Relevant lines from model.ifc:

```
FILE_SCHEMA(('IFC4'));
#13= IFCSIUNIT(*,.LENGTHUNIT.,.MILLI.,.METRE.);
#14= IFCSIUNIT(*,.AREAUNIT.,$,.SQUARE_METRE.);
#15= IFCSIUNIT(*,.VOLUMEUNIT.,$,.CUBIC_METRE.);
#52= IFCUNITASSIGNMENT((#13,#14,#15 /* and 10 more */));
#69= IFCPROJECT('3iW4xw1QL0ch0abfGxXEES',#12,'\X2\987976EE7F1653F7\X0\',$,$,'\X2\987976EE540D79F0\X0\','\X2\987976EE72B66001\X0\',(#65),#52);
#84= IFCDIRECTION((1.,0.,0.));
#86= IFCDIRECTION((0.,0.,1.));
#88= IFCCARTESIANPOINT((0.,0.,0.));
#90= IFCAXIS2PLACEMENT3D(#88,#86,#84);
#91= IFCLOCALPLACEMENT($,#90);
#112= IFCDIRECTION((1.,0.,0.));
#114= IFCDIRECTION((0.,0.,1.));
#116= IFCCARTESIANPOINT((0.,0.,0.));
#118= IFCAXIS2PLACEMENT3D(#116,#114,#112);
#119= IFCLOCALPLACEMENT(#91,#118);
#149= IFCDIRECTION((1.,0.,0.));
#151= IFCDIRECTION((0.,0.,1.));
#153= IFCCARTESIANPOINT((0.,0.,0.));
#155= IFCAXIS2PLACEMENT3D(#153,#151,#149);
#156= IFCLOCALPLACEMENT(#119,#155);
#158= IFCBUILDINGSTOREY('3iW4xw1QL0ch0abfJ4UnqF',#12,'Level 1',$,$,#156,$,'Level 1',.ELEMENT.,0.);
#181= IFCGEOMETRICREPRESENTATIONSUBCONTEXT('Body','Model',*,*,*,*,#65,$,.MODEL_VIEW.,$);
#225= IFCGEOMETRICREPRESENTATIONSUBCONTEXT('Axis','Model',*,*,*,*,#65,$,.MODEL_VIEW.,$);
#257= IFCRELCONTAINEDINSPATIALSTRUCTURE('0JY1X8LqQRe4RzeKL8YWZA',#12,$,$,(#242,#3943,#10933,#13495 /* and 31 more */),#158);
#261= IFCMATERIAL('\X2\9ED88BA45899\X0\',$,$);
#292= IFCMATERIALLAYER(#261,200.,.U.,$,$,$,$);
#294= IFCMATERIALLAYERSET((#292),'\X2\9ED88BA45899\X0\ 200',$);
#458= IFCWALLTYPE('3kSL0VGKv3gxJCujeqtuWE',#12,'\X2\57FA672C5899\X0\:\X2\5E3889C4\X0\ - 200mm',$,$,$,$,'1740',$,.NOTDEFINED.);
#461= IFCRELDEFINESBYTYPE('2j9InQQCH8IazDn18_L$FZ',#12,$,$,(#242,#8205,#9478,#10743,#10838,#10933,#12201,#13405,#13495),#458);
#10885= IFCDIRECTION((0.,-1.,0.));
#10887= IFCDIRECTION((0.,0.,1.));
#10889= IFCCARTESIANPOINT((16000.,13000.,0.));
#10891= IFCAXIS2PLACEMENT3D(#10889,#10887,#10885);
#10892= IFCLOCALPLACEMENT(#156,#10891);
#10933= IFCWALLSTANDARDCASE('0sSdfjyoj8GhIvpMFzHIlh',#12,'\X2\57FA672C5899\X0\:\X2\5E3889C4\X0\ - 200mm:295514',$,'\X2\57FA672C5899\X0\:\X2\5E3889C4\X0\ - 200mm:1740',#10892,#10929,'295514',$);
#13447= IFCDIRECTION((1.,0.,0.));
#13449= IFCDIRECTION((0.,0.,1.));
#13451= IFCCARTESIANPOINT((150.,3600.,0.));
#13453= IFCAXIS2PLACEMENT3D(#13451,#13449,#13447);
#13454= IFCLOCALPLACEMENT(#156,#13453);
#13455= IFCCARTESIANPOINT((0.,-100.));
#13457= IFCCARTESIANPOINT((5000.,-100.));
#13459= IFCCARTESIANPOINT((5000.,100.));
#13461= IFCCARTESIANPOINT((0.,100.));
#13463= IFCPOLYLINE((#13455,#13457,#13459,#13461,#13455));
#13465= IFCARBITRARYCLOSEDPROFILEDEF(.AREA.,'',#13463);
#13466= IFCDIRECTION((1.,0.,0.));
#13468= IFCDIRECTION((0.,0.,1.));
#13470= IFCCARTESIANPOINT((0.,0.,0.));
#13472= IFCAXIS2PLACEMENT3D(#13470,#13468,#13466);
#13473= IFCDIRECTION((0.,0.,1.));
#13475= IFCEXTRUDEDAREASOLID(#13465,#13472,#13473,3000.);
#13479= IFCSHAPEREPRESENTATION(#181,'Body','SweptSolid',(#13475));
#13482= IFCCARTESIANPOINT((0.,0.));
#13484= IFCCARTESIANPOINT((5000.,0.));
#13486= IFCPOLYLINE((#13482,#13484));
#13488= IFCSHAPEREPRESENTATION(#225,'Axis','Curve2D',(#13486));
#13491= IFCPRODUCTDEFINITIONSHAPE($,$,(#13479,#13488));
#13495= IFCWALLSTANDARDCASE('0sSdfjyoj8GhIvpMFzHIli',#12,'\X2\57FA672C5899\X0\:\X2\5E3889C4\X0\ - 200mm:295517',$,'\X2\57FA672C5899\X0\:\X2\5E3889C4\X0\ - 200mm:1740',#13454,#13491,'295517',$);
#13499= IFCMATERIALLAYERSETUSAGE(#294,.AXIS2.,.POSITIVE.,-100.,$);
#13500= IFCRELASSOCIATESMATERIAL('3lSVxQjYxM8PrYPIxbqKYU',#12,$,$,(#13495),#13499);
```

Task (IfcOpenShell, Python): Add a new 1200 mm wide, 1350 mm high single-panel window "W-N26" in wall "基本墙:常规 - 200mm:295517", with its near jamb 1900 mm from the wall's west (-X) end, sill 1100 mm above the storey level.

```python
import numpy as np
import ifcopenshell
import ifcopenshell.api.feature
import ifcopenshell.api.geometry
import ifcopenshell.api.root
import ifcopenshell.api.spatial
import ifcopenshell.geom
import ifcopenshell.util.element
import ifcopenshell.util.placement
import ifcopenshell.util.representation
import ifcopenshell.util.shape
import ifcopenshell.util.unit

model = ifcopenshell.open("model.ifc")
unit_scale = ifcopenshell.util.unit.calculate_unit_scale(model)
settings = ifcopenshell.geom.settings()


def volume(element):
    """Net volume in cubic metres, openings subtracted."""
    shape = ifcopenshell.geom.create_shape(settings, element)
    return ifcopenshell.util.shape.get_volume(shape.geometry)


wall = model.by_id(13495)
storey = ifcopenshell.util.element.get_container(wall, ifc_class="IfcBuildingStorey")
context = ifcopenshell.util.representation.get_context(model, "Model", "Body", "MODEL_VIEW")
before = volume(wall)

width, height, from_end, sill = 1.2, 1.35, 1.9, 1.1  # metres

# The wall runs along its own X axis, and the end named is its -X end.
wall_shape = ifcopenshell.geom.create_shape(settings, wall)
x, y, z = ifcopenshell.util.shape.get_vertices(wall_shape.geometry).T
start = x.min() + from_end
face, thickness = float(y.min()), float(y.max() - y.min())
wall_matrix = ifcopenshell.util.placement.get_local_placement(wall.ObjectPlacement)
level = ifcopenshell.util.placement.get_local_placement(storey.ObjectPlacement)[2, 3]


def in_wall(x, y):
    """Placement at x, y metres in the wall's axes, at sill height."""
    matrix = wall_matrix.copy()
    matrix[:, 3] = wall_matrix @ np.array([x / unit_scale, y / unit_scale, 0.0, 1.0])
    matrix[2, 3] = level + sill / unit_scale
    return matrix


# Opening: a box that overshoots both wall faces by 50 mm.
opening = ifcopenshell.api.root.create_entity(model, ifc_class="IfcOpeningElement", predefined_type="OPENING")
box = ifcopenshell.api.geometry.add_wall_representation(
    model, context=context, length=width, height=height, thickness=thickness + 0.1
)
ifcopenshell.api.geometry.assign_representation(model, product=opening, representation=box)
ifcopenshell.api.geometry.edit_object_placement(model, product=opening, matrix=in_wall(start, face - 0.05), is_si=False)
ifcopenshell.api.feature.add_feature(model, feature=opening, element=wall)

window = ifcopenshell.api.root.create_entity(model, ifc_class="IfcWindow", name="W-N26", predefined_type="WINDOW")
window.OverallWidth, window.OverallHeight = width / unit_scale, height / unit_scale
window.PartitioningType = "SINGLE_PANEL"
body = ifcopenshell.api.geometry.add_window_representation(
    model,
    context=context,
    overall_width=window.OverallWidth,
    overall_height=window.OverallHeight,
    partition_type="SINGLE_PANEL",
)
ifcopenshell.api.geometry.assign_representation(model, product=window, representation=body)
ifcopenshell.api.spatial.assign_container(model, products=[window], relating_structure=storey)
ifcopenshell.api.feature.add_filling(model, opening=opening, element=window)

# Centre the window in the wall's thickness.
ifcopenshell.api.geometry.edit_object_placement(model, product=window, matrix=in_wall(start, face), is_si=False)
window_shape = ifcopenshell.geom.create_shape(settings, window)
depth = ifcopenshell.util.shape.get_vertices(window_shape.geometry)[:, 1]
offset = face + thickness / 2 - (depth.min() + depth.max()) / 2
ifcopenshell.api.geometry.edit_object_placement(model, product=window, matrix=in_wall(start, offset), is_si=False)

after = volume(wall)

print(f"wall volume {before:.3f} -> {after:.3f} m3")

model.write("model_v2.ifc")
```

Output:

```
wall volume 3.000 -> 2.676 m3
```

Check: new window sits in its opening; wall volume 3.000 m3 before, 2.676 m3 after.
